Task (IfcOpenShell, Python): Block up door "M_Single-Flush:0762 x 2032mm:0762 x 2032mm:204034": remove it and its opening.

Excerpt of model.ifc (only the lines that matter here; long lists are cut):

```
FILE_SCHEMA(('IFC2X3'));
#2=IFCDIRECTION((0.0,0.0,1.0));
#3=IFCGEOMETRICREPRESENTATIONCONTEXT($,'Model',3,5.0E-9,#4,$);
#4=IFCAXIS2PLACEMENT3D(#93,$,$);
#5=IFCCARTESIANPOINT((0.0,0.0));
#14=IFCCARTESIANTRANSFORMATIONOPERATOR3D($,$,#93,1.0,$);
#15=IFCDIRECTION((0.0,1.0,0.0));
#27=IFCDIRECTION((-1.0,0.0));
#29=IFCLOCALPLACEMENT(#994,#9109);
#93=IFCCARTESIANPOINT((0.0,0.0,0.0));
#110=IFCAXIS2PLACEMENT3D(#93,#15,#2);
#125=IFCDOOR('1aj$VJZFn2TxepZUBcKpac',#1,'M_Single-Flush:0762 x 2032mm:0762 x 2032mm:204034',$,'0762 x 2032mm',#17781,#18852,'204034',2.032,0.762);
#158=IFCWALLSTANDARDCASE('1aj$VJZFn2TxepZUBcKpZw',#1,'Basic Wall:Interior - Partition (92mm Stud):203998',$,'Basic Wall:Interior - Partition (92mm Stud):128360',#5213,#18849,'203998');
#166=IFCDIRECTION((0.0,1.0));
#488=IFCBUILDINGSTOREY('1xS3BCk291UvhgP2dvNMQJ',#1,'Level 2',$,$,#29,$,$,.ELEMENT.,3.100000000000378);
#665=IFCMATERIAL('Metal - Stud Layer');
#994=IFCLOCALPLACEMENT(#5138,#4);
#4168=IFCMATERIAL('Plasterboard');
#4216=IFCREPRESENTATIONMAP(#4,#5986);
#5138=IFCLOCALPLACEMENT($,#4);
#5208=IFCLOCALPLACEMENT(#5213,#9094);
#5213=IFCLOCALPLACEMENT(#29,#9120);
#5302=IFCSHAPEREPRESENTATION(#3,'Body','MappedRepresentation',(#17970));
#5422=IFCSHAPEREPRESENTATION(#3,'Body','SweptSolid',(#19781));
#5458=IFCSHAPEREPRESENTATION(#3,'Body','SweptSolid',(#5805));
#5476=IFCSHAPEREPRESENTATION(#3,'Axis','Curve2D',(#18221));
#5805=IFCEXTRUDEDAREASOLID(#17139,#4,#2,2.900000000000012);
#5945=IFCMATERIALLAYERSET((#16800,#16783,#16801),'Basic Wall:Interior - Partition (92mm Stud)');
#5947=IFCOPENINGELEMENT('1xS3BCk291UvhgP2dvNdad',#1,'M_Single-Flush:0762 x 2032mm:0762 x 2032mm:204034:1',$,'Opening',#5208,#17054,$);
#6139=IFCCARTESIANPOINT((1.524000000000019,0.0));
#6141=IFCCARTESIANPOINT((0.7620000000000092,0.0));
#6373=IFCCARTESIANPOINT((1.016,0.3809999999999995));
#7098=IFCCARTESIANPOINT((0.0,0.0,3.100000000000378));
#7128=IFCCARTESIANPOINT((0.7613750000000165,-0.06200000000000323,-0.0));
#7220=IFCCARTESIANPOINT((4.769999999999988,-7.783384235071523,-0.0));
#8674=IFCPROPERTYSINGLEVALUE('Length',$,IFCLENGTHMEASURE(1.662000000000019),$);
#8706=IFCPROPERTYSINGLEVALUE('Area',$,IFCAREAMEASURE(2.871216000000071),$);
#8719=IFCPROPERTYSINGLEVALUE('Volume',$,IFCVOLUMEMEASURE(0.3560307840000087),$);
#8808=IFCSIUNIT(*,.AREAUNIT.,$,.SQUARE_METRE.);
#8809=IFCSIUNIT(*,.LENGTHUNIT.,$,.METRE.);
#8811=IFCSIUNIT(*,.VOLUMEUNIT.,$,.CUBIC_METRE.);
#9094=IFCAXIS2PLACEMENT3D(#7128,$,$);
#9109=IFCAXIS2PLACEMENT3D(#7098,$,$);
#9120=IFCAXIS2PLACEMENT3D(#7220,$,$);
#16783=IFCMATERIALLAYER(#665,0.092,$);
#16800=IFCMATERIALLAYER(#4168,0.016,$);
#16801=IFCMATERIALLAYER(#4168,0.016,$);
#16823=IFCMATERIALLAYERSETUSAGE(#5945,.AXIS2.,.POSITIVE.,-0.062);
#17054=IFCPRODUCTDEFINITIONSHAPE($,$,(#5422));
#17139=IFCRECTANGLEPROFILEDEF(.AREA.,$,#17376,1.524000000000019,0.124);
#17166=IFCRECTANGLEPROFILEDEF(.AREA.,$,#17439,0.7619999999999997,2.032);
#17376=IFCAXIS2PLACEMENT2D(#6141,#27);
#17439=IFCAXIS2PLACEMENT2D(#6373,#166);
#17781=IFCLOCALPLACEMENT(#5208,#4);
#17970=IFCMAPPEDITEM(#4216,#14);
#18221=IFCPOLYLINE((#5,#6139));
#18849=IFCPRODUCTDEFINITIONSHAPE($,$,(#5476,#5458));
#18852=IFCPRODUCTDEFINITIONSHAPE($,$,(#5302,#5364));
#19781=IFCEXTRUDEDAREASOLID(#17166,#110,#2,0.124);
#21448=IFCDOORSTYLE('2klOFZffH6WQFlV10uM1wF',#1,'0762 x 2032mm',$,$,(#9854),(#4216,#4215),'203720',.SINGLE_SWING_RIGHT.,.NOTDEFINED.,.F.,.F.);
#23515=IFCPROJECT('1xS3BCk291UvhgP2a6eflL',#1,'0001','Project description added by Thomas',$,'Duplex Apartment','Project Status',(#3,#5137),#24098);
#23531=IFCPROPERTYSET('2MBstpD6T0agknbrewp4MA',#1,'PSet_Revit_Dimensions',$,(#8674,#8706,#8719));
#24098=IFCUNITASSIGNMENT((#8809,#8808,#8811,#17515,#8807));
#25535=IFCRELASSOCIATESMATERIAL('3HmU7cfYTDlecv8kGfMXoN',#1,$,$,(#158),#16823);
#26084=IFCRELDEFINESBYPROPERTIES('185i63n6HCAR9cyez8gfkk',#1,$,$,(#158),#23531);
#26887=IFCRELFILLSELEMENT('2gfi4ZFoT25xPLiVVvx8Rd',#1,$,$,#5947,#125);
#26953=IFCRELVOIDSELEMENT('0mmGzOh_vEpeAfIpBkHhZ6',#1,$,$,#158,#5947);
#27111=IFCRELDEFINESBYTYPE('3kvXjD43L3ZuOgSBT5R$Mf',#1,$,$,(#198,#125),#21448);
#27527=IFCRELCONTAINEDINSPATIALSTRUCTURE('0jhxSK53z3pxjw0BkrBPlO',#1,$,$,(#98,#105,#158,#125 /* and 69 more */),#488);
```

```python
import ifcopenshell
import ifcopenshell.api.feature
import ifcopenshell.api.pset
import ifcopenshell.api.root
import ifcopenshell.geom
import ifcopenshell.util.element
import ifcopenshell.util.shape
import ifcopenshell.util.unit

model = ifcopenshell.open("model.ifc")
area_scale = ifcopenshell.util.unit.calculate_unit_scale(model, "AREAUNIT")
volume_scale = ifcopenshell.util.unit.calculate_unit_scale(model, "VOLUMEUNIT")
settings = ifcopenshell.geom.settings()


def volume(element):
    """Net volume in cubic metres, openings subtracted."""
    shape = ifcopenshell.geom.create_shape(settings, element)
    return ifcopenshell.util.shape.get_volume(shape.geometry)


door = model.by_id(125)
opening = door.FillsVoids[0].RelatingOpeningElement
wall = opening.VoidsElements[0].RelatingBuildingElement
before = volume(wall)

ifcopenshell.api.root.remove_product(model, product=door)
ifcopenshell.api.feature.remove_feature(model, feature=opening)

after = volume(wall)
thickness = 0.124  # wall thickness in metres

# Update the wall's stored quantities.
pset = model.by_id(ifcopenshell.util.element.get_pset(wall, "PSet_Revit_Dimensions", should_inherit=False)["id"])
ifcopenshell.api.pset.edit_pset(model, pset=pset, properties={
    "Area": model.create_entity("IfcAreaMeasure", after / thickness / area_scale),
    "Volume": model.create_entity("IfcVolumeMeasure", after / volume_scale),
})

print(f"wall volume {before:.3f} -> {after:.3f} m3")

model.write("model-out.ifc")
```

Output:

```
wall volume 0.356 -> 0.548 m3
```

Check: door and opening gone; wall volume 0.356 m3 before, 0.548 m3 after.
